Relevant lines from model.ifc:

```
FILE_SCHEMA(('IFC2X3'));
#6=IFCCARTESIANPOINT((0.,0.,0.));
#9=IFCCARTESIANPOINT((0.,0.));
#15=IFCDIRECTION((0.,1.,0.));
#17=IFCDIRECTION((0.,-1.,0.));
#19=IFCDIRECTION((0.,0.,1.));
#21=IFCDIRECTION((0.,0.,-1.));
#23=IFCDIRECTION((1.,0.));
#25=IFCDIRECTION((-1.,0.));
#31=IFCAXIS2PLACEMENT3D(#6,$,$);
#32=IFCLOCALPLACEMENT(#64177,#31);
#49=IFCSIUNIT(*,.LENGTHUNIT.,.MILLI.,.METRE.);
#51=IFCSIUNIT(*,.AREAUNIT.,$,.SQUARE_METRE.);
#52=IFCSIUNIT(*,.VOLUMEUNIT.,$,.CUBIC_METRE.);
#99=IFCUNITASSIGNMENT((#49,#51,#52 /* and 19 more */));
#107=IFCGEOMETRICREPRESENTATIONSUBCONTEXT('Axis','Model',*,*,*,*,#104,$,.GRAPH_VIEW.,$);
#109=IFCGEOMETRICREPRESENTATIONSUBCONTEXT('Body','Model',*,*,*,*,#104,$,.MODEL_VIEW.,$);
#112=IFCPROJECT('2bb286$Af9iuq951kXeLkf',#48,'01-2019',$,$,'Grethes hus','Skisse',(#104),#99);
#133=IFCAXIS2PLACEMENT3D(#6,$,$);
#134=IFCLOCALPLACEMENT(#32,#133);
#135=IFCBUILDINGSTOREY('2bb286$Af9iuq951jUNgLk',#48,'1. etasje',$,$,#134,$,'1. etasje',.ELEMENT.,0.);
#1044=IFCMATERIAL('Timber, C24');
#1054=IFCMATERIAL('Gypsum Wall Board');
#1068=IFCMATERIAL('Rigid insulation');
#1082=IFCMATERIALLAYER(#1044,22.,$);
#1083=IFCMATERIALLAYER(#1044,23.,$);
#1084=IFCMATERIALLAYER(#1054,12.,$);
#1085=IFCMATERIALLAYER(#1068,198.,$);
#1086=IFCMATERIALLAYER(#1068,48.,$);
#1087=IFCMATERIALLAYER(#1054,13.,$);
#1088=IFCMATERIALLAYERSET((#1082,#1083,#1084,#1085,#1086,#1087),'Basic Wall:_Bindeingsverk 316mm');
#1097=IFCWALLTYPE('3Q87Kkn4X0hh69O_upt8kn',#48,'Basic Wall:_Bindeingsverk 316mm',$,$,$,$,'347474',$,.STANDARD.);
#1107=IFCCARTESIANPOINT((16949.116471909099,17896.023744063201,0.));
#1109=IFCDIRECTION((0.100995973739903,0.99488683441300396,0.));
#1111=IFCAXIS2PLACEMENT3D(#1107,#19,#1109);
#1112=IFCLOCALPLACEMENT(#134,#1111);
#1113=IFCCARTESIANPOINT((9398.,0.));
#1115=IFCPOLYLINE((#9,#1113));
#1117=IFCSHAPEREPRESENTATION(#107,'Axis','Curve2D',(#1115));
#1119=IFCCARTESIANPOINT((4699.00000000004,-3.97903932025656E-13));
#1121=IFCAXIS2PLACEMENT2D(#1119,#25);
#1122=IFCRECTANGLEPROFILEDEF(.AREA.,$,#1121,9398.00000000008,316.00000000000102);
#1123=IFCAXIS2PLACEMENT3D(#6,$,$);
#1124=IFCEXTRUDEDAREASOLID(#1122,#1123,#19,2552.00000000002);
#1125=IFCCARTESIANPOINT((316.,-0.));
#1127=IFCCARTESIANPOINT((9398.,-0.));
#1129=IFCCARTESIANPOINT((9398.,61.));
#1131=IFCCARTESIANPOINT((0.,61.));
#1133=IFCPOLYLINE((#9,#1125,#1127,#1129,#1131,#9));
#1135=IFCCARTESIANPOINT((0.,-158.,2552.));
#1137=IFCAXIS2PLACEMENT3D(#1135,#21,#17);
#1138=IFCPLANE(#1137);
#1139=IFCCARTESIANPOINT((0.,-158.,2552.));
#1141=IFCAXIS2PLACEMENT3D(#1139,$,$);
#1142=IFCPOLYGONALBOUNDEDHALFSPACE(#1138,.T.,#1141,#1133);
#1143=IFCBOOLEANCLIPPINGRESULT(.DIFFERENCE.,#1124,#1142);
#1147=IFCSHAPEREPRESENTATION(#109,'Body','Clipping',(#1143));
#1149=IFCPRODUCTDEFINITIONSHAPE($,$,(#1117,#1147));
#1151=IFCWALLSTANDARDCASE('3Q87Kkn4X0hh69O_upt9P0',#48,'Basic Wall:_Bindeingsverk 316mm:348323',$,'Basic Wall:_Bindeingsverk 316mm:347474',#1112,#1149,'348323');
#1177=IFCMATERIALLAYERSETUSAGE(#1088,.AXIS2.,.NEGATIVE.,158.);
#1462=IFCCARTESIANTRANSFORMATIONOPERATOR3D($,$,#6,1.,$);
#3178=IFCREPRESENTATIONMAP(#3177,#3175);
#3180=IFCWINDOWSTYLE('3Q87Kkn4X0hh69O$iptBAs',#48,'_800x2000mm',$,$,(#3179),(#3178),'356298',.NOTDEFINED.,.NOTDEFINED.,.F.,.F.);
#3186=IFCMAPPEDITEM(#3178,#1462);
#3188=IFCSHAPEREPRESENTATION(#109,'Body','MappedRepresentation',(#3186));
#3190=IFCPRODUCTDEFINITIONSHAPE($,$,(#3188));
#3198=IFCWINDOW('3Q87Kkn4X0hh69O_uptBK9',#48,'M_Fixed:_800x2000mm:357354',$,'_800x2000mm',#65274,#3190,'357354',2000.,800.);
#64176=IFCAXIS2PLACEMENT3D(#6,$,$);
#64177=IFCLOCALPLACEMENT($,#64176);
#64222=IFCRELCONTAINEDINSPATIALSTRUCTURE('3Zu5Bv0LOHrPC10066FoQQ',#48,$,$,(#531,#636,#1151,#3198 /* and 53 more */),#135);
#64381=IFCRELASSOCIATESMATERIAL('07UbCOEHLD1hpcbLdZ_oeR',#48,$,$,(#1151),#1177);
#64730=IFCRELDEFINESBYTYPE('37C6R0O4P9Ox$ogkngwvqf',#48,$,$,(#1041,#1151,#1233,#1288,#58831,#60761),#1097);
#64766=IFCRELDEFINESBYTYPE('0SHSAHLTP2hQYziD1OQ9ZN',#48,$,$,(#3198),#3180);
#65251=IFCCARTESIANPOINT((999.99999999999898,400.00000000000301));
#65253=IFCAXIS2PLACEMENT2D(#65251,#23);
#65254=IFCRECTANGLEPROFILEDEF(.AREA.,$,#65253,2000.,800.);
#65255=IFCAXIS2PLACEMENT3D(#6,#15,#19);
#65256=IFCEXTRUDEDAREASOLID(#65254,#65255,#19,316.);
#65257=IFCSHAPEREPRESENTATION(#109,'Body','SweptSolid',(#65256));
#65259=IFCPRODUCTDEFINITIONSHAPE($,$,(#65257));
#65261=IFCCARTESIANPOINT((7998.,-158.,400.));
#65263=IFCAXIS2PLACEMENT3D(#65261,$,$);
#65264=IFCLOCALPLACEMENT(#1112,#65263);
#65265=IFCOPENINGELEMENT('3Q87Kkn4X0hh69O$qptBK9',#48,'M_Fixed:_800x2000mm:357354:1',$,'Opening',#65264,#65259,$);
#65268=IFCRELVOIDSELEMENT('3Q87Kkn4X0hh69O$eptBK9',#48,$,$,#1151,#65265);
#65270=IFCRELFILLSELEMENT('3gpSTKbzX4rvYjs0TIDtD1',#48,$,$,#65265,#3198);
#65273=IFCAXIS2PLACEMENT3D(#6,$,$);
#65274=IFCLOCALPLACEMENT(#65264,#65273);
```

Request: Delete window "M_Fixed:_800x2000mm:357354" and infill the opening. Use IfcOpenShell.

```python
import ifcopenshell
import ifcopenshell.api.feature
import ifcopenshell.api.root
import ifcopenshell.geom
import ifcopenshell.util.shape

model = ifcopenshell.open("model.ifc")
settings = ifcopenshell.geom.settings()


def volume(element):
    """Net volume in cubic metres, openings subtracted."""
    shape = ifcopenshell.geom.create_shape(settings, element)
    return ifcopenshell.util.shape.get_volume(shape.geometry)


window = model.by_guid("3Q87Kkn4X0hh69O_uptBK9")
opening = window.FillsVoids[0].RelatingOpeningElement
wall = opening.VoidsElements[0].RelatingBuildingElement
before = volume(wall)

ifcopenshell.api.root.remove_product(model, product=window)
ifcopenshell.api.feature.remove_feature(model, feature=opening)

after = volume(wall)

print(f"wall volume {before:.3f} -> {after:.3f} m3")

model.write("model_v2.ifc")
```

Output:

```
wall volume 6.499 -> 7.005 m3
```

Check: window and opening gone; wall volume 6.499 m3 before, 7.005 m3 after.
